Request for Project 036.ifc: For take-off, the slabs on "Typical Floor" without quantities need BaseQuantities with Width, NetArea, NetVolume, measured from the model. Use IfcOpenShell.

First a look at what the model holds.

```python
import ifcopenshell
import ifcopenshell.util.element
import ifcopenshell.util.unit

model = ifcopenshell.open("Project 036.ifc")
print(model.schema)
for unit_type in ("LENGTHUNIT", "AREAUNIT", "VOLUMEUNIT"):
    print(unit_type, ifcopenshell.util.unit.calculate_unit_scale(model, unit_type))
storey = next(s for s in model.by_type("IfcBuildingStorey") if s.Name == "Typical Floor")
slabs = [e for e in ifcopenshell.util.element.get_decomposition(storey) if e.is_a("IfcSlab")]
for e in sorted(slabs, key=lambda e: e.id()):
    print(e.id(), e.is_a(), e.Name, list(ifcopenshell.util.element.get_psets(e, qtos_only=True)), sep=" | ")
```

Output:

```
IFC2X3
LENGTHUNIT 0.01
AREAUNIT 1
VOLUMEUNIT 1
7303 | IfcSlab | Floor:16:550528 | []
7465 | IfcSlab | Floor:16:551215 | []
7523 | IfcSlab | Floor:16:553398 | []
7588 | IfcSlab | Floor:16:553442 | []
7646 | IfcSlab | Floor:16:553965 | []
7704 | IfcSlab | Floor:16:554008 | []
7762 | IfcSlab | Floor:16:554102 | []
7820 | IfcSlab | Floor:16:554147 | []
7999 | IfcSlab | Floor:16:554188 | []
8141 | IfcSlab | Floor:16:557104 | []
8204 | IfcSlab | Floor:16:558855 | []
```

```python
import ifcopenshell
import ifcopenshell.api.pset
import ifcopenshell.geom
import ifcopenshell.util.element
import ifcopenshell.util.shape
import ifcopenshell.util.unit

model = ifcopenshell.open("Project 036.ifc")
unit_scale = ifcopenshell.util.unit.calculate_unit_scale(model)
area_scale = ifcopenshell.util.unit.calculate_unit_scale(model, "AREAUNIT")
volume_scale = ifcopenshell.util.unit.calculate_unit_scale(model, "VOLUMEUNIT")
settings = ifcopenshell.geom.settings()

storey = next(s for s in model.by_type("IfcBuildingStorey") if s.Name == "Typical Floor")
slabs = [e for e in ifcopenshell.util.element.get_decomposition(storey) if e.is_a("IfcSlab")]

for e in sorted(slabs, key=lambda e: e.id()):
    if ifcopenshell.util.element.get_psets(e, qtos_only=True, should_inherit=False):
        continue
    # Geometry comes back in metres, in the element's own axes.
    shape = ifcopenshell.geom.create_shape(settings, e)
    values = {
        "Width": ifcopenshell.util.shape.get_z(shape.geometry) / unit_scale,
        "NetArea": ifcopenshell.util.shape.get_footprint_area(shape.geometry) / area_scale,
        "NetVolume": ifcopenshell.util.shape.get_volume(shape.geometry) / volume_scale,
    }
    qto = ifcopenshell.api.pset.add_qto(model, product=e, name="BaseQuantities")
    ifcopenshell.api.pset.edit_qto(model, qto=qto, properties=values)
    print(e.id(), {k: round(v, 3) for k, v in values.items()})

model.write("Project 036_v2.ifc")
```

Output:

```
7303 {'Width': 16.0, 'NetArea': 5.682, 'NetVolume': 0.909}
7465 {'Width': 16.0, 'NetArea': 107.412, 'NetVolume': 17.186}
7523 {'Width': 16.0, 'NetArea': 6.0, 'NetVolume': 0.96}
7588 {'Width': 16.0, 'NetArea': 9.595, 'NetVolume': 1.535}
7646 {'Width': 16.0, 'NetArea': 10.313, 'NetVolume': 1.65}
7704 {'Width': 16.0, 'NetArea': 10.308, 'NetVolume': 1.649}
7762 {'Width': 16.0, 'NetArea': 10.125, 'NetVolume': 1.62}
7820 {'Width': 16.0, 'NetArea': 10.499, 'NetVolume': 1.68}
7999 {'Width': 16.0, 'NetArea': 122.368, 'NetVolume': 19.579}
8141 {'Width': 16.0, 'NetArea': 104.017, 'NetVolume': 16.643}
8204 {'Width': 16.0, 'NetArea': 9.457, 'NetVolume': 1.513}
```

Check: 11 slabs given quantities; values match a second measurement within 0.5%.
